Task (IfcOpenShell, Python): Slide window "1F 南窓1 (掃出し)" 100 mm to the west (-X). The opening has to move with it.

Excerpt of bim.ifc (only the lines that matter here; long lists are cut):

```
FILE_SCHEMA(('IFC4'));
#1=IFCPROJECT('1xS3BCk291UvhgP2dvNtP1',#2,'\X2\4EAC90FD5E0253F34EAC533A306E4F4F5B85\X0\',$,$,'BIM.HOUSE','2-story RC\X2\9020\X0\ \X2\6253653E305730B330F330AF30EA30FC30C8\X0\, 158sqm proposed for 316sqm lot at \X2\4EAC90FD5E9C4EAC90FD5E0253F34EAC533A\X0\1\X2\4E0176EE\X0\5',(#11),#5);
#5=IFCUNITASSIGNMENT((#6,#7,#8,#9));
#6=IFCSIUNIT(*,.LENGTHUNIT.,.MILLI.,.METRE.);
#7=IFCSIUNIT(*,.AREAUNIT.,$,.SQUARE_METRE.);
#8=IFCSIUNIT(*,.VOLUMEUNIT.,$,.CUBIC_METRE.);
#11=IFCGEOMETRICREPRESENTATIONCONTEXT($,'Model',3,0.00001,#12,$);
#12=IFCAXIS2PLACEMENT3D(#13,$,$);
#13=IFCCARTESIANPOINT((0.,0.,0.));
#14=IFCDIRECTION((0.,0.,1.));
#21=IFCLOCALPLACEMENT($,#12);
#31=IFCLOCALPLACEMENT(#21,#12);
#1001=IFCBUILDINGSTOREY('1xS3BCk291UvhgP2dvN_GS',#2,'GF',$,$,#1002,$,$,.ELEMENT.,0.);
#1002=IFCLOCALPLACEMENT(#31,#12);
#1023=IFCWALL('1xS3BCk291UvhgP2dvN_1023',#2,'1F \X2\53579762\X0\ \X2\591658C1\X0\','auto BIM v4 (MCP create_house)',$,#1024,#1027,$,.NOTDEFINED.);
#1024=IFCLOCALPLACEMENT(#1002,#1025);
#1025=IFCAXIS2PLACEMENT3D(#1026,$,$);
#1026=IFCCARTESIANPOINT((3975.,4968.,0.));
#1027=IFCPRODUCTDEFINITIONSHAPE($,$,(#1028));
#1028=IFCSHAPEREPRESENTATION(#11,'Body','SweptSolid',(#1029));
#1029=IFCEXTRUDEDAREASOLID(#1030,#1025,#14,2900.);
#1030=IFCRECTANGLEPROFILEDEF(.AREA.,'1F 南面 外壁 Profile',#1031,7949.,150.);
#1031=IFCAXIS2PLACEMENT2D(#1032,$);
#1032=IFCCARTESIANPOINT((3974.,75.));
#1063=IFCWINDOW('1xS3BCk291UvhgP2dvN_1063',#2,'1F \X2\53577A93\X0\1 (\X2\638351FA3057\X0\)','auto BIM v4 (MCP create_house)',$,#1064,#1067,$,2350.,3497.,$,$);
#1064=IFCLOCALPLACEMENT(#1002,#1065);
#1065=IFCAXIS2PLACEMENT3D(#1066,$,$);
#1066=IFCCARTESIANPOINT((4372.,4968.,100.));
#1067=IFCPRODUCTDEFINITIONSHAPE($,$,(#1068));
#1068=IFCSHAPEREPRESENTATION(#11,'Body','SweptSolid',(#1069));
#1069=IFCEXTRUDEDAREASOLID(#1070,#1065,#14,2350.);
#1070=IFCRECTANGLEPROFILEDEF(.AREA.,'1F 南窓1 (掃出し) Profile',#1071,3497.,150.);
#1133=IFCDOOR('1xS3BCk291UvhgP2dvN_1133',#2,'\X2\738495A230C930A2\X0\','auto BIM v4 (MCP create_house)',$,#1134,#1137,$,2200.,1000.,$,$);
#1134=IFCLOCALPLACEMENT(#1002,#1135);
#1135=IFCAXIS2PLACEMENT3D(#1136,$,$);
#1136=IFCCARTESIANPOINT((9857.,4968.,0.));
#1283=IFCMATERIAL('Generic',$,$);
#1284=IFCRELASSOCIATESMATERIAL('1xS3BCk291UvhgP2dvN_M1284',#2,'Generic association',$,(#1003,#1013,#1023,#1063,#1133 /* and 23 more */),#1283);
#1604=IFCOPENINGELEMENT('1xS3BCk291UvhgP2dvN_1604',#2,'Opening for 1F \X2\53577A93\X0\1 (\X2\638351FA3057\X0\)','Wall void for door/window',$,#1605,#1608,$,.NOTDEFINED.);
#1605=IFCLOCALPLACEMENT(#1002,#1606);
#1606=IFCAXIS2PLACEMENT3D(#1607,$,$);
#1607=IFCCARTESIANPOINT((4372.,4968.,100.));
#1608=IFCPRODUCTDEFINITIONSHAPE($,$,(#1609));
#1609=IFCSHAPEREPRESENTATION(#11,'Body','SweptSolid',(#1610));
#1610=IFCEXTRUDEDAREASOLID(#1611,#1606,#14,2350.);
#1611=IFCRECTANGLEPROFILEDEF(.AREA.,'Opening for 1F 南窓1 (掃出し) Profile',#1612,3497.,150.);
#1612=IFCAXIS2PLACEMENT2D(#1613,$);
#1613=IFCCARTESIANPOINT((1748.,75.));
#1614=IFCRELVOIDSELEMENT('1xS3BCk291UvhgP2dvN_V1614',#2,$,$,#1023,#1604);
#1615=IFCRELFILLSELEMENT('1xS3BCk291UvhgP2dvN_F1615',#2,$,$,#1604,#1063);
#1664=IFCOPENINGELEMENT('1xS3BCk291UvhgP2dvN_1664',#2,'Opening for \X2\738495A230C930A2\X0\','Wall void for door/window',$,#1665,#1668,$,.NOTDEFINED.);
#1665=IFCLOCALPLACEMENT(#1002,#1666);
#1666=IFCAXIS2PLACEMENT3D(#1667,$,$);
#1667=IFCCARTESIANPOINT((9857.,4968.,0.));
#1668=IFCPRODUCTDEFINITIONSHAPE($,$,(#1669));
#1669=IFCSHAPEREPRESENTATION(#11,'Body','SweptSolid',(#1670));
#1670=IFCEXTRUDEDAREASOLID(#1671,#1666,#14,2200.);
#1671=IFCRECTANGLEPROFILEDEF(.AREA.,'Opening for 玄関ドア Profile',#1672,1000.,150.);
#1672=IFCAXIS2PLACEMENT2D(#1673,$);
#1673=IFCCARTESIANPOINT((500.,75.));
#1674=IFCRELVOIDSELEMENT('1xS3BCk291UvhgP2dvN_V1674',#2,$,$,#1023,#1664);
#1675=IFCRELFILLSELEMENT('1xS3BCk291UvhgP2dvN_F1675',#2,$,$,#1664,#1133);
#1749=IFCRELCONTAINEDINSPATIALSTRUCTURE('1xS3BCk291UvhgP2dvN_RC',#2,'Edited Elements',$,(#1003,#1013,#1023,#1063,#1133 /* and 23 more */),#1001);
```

```python
import ifcopenshell
import ifcopenshell.api.geometry
import ifcopenshell.util.placement

model = ifcopenshell.open("bim.ifc")

window = model.by_guid("1xS3BCk291UvhgP2dvN_1063")
opening = window.FillsVoids[0].RelatingOpeningElement
wall = opening.VoidsElements[0].RelatingBuildingElement

wall_matrix = ifcopenshell.util.placement.get_local_placement(wall.ObjectPlacement)
shift = wall_matrix[:3, 0] * -100.0
before = ifcopenshell.util.placement.get_local_placement(window.ObjectPlacement)[:3, 3].copy()

# The window is not placed relative to its opening, so move both.
for product in (opening, window):
    matrix = ifcopenshell.util.placement.get_local_placement(product.ObjectPlacement)
    matrix[:3, 3] += shift
    ifcopenshell.api.geometry.edit_object_placement(model, product=product, matrix=matrix, is_si=False)

after = ifcopenshell.util.placement.get_local_placement(window.ObjectPlacement)[:3, 3]
print("window moved by", (after - before).round(3) + 0.0)

model.write("bim_updated.ifc")
```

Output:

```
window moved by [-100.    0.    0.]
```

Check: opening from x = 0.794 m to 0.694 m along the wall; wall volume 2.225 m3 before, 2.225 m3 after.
